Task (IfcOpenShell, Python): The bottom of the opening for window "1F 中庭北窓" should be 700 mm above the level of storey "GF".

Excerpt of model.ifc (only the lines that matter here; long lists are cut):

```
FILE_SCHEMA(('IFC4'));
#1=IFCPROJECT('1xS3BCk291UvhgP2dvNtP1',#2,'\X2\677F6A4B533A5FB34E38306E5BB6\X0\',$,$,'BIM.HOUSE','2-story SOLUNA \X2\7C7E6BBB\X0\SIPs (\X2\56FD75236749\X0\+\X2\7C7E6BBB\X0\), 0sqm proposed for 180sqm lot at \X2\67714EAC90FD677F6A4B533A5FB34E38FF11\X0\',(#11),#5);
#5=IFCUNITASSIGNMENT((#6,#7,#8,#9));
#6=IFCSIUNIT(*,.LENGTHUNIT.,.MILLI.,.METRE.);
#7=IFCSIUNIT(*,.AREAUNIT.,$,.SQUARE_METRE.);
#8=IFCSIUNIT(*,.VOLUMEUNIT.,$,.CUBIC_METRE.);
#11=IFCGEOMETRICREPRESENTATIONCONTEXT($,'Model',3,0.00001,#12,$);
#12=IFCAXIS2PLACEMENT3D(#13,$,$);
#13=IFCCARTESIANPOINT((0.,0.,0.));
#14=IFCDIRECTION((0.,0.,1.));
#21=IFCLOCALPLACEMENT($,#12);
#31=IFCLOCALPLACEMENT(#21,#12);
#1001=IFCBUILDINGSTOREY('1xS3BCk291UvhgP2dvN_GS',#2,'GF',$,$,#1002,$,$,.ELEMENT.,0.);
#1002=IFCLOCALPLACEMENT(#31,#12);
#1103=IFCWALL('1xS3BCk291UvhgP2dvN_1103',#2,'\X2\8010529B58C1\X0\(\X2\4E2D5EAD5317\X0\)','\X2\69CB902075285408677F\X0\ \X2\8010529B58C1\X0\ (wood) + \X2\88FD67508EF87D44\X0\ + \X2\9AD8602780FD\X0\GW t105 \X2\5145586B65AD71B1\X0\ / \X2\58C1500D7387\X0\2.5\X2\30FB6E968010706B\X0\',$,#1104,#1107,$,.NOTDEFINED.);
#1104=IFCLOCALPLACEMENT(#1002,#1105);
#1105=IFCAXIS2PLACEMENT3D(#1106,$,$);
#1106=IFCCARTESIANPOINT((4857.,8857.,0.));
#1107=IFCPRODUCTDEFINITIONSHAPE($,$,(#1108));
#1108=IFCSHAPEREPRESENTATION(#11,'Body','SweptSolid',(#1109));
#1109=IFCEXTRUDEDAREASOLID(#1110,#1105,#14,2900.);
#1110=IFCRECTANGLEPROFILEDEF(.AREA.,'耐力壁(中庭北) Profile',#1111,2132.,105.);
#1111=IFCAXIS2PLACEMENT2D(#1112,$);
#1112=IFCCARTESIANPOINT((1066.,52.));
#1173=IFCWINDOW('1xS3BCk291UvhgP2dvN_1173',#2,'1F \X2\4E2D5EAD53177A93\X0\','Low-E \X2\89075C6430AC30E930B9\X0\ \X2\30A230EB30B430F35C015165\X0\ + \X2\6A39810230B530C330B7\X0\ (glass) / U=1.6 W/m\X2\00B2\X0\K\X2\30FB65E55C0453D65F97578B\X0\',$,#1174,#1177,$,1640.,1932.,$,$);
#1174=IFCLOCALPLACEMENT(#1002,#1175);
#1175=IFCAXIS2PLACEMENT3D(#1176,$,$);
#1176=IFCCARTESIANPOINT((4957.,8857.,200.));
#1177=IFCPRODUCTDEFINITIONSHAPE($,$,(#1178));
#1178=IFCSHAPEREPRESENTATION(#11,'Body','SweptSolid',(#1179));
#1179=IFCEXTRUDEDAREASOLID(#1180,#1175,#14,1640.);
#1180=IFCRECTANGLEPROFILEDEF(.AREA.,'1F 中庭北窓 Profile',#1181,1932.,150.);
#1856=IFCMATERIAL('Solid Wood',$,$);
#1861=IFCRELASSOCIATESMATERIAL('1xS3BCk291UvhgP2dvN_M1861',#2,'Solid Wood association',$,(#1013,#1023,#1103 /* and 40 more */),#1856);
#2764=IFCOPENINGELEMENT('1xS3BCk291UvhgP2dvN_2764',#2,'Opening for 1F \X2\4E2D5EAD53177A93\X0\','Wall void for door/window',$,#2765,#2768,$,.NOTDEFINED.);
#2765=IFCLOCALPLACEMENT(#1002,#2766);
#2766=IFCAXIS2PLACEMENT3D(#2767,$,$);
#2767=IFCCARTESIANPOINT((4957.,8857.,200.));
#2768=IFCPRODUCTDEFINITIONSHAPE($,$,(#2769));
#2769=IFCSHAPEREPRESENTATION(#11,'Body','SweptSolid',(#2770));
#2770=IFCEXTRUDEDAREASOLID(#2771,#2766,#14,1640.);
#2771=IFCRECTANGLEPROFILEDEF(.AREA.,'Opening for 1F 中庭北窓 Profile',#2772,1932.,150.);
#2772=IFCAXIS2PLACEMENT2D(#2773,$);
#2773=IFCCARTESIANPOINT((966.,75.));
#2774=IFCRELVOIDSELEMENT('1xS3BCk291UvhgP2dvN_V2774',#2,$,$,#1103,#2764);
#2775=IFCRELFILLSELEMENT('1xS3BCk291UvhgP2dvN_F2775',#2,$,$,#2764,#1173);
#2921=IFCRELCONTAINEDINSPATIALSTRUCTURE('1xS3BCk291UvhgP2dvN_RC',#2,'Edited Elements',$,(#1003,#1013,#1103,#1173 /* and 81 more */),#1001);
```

```python
import numpy as np
import ifcopenshell
import ifcopenshell.api.geometry
import ifcopenshell.geom
import ifcopenshell.util.element
import ifcopenshell.util.placement
import ifcopenshell.util.shape
import ifcopenshell.util.unit

model = ifcopenshell.open("model.ifc")
unit_scale = ifcopenshell.util.unit.calculate_unit_scale(model)

window = model.by_guid("1xS3BCk291UvhgP2dvN_1173")
opening = window.FillsVoids[0].RelatingOpeningElement
storey = ifcopenshell.util.element.get_container(window, ifc_class="IfcBuildingStorey")
level = ifcopenshell.util.placement.get_local_placement(storey.ObjectPlacement)[2, 3]

# The opening's origin need not be at the sill, so measure its lowest point.
shape = ifcopenshell.geom.create_shape(ifcopenshell.geom.settings(), opening)
bottom = ifcopenshell.util.shape.get_shape_bottom_elevation(shape, shape.geometry) / unit_scale
dz = level + 0.7 / unit_scale - bottom

shift = np.array([0.0, 0.0, dz])
# The window is not placed relative to its opening, so move both.
for product in (opening, window):
    matrix = ifcopenshell.util.placement.get_local_placement(product.ObjectPlacement)
    matrix[:3, 3] += shift
    ifcopenshell.api.geometry.edit_object_placement(model, product=product, matrix=matrix, is_si=False)

print(f"moved by {dz * unit_scale:+.3f} m")

model.write("model_updated.ifc")
```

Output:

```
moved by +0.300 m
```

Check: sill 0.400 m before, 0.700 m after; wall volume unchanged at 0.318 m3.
